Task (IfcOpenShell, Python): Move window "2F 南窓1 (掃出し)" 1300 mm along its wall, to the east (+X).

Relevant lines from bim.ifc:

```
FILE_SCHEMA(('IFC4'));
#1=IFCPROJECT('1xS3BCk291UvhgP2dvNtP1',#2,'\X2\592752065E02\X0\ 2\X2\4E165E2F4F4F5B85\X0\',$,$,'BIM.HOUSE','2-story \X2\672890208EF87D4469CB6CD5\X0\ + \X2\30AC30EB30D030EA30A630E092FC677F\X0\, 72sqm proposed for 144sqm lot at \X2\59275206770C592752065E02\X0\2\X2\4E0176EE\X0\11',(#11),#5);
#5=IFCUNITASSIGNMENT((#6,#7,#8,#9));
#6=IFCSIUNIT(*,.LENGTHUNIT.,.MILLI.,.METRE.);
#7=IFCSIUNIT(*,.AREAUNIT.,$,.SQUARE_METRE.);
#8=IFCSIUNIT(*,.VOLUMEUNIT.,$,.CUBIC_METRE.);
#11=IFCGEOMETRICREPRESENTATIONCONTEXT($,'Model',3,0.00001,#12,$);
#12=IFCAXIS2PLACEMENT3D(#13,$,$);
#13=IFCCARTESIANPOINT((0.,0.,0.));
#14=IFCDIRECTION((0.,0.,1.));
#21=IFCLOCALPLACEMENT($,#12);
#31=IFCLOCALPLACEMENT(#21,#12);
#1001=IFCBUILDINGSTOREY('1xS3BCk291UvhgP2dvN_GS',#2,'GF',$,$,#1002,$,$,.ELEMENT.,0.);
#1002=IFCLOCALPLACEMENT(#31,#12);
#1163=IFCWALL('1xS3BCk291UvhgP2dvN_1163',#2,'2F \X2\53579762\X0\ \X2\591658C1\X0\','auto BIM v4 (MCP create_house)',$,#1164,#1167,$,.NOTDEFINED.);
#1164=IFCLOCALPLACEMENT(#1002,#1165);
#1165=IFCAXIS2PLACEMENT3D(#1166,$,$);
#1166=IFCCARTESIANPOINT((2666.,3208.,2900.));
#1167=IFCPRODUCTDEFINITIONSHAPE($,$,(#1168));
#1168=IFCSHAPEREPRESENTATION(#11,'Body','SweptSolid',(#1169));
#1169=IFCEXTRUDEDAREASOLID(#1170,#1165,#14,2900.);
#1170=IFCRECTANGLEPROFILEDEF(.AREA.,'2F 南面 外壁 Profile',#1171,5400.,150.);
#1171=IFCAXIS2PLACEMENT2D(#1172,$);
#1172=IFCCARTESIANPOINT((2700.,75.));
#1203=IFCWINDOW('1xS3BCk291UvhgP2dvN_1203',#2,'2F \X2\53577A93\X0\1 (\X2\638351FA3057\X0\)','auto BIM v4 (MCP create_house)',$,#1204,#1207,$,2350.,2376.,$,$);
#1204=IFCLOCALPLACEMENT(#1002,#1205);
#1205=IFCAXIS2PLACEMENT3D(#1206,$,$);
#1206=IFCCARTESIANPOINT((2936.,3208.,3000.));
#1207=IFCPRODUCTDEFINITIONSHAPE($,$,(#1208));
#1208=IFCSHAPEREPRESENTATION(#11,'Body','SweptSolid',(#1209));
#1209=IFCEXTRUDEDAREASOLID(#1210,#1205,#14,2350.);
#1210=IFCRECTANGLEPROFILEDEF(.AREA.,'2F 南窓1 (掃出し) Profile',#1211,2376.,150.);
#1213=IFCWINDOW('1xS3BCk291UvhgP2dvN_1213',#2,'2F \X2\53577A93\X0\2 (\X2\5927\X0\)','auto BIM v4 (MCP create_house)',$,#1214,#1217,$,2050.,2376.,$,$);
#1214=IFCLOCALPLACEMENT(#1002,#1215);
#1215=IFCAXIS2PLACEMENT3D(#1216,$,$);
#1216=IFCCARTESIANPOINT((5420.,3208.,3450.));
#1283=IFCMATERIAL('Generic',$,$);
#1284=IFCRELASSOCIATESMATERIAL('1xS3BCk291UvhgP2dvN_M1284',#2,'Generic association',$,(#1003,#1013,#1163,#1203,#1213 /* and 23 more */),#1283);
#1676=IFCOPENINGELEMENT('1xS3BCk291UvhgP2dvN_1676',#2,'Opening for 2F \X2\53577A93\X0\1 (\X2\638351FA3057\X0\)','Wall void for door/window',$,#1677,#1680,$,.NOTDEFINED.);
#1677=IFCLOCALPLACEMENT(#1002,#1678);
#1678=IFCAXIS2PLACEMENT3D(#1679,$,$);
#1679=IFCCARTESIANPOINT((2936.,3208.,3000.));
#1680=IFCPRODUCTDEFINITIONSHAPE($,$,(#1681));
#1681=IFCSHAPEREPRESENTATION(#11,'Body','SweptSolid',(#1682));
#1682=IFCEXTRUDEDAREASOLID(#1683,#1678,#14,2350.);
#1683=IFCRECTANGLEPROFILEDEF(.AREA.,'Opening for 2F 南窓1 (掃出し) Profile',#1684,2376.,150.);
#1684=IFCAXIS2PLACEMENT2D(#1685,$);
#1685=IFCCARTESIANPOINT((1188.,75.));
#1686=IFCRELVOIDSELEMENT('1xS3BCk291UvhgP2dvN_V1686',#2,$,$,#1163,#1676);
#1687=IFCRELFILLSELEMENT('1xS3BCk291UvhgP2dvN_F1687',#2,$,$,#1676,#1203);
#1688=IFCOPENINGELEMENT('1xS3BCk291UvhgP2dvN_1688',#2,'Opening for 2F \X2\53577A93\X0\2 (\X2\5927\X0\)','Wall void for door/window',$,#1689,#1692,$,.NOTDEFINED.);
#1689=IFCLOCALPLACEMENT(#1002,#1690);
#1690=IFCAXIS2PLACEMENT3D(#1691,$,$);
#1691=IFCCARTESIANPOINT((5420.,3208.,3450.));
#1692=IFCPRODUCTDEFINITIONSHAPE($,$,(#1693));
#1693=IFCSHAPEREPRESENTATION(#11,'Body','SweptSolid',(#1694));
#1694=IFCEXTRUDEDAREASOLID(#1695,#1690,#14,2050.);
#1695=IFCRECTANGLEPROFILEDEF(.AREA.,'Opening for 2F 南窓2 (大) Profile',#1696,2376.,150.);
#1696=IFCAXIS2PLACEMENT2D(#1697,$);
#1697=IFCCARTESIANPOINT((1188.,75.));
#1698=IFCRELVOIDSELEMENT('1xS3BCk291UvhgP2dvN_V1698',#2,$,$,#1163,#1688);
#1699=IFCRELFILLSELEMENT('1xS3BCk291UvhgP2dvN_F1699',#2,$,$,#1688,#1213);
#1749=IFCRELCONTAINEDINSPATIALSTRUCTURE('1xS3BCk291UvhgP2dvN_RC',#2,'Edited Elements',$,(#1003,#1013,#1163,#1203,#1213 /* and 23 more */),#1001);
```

```python
import ifcopenshell
import ifcopenshell.api.geometry
import ifcopenshell.util.placement

model = ifcopenshell.open("bim.ifc")

window = model.by_guid("1xS3BCk291UvhgP2dvN_1203")
opening = window.FillsVoids[0].RelatingOpeningElement
wall = opening.VoidsElements[0].RelatingBuildingElement

wall_matrix = ifcopenshell.util.placement.get_local_placement(wall.ObjectPlacement)
shift = wall_matrix[:3, 0] * 1300.0
before = ifcopenshell.util.placement.get_local_placement(window.ObjectPlacement)[:3, 3].copy()

# The window is not placed relative to its opening, so move both.
for product in (opening, window):
    matrix = ifcopenshell.util.placement.get_local_placement(product.ObjectPlacement)
    matrix[:3, 3] += shift
    ifcopenshell.api.geometry.edit_object_placement(model, product=product, matrix=matrix, is_si=False)

after = ifcopenshell.util.placement.get_local_placement(window.ObjectPlacement)[:3, 3]
print("window moved by", (after - before).round(3) + 0.0)

model.write("bim_rev.ifc")
```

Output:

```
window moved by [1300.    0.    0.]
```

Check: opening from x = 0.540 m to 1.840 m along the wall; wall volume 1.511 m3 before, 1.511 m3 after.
